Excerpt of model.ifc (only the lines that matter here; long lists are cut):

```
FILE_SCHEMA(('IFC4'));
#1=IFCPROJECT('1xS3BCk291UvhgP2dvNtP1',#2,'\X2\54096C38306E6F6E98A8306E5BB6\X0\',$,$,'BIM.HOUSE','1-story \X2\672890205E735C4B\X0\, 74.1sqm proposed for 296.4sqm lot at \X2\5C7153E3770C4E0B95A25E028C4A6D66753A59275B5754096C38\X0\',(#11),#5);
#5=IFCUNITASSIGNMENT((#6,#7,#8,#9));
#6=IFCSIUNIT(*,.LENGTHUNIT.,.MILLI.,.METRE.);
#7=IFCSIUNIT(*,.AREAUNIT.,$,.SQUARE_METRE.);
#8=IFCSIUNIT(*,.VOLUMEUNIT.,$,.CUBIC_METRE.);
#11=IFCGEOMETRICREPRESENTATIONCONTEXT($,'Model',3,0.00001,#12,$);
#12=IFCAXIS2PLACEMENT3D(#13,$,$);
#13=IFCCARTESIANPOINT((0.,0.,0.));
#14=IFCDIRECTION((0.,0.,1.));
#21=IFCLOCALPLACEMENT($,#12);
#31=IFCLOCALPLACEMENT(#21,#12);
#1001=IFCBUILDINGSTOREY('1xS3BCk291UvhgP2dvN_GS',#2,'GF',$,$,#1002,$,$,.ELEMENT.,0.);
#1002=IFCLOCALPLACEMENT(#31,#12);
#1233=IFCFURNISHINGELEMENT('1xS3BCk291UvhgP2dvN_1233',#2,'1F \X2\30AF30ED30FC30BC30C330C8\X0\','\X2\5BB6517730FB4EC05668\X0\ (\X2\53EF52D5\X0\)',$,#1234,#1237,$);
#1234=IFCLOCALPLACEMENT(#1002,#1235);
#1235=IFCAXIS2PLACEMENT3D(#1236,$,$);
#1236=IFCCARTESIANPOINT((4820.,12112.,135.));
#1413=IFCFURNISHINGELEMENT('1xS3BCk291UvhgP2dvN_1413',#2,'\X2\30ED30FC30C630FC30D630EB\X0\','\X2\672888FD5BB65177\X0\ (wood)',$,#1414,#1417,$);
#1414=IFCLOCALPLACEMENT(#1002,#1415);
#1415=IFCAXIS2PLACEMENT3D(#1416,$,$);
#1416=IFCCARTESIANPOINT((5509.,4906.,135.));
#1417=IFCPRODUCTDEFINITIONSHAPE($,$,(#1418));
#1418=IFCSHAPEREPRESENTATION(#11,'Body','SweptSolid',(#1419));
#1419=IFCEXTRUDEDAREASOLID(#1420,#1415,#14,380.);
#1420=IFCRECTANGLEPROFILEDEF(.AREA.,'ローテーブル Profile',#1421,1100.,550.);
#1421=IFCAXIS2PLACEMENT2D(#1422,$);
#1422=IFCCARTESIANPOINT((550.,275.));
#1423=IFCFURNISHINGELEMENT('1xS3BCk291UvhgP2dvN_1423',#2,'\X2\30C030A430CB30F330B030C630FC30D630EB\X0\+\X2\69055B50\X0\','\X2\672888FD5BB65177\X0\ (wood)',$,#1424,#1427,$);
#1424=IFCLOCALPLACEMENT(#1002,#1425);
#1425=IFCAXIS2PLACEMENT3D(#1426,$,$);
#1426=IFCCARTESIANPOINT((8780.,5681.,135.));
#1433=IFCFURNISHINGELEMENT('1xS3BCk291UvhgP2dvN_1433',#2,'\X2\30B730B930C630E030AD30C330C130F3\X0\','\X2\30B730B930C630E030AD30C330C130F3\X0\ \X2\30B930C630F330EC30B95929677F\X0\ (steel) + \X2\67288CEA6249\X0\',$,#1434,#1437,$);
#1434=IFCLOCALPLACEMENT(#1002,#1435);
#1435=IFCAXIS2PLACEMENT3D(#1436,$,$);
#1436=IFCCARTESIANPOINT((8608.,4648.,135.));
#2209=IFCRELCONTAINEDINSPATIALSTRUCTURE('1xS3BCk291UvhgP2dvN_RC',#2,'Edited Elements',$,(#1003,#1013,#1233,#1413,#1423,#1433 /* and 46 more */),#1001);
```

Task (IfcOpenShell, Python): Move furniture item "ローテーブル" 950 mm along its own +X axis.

```python
import ifcopenshell
import ifcopenshell.api.geometry
import ifcopenshell.util.placement
import ifcopenshell.util.unit

model = ifcopenshell.open("model.ifc")
unit_scale = ifcopenshell.util.unit.calculate_unit_scale(model)

item = model.by_guid("1xS3BCk291UvhgP2dvN_1413")
matrix = ifcopenshell.util.placement.get_local_placement(item.ObjectPlacement)
matrix[:3, 3] += matrix[:3, 0] * 0.95 / unit_scale
ifcopenshell.api.geometry.edit_object_placement(model, product=item, matrix=matrix, is_si=False)

print(ifcopenshell.util.placement.get_local_placement(item.ObjectPlacement).round(3) + 0.0)

model.write("model_updated.ifc")
```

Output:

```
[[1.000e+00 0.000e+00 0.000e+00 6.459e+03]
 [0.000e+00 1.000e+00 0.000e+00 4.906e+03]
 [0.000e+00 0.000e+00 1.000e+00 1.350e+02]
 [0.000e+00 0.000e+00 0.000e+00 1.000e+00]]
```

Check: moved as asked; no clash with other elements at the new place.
